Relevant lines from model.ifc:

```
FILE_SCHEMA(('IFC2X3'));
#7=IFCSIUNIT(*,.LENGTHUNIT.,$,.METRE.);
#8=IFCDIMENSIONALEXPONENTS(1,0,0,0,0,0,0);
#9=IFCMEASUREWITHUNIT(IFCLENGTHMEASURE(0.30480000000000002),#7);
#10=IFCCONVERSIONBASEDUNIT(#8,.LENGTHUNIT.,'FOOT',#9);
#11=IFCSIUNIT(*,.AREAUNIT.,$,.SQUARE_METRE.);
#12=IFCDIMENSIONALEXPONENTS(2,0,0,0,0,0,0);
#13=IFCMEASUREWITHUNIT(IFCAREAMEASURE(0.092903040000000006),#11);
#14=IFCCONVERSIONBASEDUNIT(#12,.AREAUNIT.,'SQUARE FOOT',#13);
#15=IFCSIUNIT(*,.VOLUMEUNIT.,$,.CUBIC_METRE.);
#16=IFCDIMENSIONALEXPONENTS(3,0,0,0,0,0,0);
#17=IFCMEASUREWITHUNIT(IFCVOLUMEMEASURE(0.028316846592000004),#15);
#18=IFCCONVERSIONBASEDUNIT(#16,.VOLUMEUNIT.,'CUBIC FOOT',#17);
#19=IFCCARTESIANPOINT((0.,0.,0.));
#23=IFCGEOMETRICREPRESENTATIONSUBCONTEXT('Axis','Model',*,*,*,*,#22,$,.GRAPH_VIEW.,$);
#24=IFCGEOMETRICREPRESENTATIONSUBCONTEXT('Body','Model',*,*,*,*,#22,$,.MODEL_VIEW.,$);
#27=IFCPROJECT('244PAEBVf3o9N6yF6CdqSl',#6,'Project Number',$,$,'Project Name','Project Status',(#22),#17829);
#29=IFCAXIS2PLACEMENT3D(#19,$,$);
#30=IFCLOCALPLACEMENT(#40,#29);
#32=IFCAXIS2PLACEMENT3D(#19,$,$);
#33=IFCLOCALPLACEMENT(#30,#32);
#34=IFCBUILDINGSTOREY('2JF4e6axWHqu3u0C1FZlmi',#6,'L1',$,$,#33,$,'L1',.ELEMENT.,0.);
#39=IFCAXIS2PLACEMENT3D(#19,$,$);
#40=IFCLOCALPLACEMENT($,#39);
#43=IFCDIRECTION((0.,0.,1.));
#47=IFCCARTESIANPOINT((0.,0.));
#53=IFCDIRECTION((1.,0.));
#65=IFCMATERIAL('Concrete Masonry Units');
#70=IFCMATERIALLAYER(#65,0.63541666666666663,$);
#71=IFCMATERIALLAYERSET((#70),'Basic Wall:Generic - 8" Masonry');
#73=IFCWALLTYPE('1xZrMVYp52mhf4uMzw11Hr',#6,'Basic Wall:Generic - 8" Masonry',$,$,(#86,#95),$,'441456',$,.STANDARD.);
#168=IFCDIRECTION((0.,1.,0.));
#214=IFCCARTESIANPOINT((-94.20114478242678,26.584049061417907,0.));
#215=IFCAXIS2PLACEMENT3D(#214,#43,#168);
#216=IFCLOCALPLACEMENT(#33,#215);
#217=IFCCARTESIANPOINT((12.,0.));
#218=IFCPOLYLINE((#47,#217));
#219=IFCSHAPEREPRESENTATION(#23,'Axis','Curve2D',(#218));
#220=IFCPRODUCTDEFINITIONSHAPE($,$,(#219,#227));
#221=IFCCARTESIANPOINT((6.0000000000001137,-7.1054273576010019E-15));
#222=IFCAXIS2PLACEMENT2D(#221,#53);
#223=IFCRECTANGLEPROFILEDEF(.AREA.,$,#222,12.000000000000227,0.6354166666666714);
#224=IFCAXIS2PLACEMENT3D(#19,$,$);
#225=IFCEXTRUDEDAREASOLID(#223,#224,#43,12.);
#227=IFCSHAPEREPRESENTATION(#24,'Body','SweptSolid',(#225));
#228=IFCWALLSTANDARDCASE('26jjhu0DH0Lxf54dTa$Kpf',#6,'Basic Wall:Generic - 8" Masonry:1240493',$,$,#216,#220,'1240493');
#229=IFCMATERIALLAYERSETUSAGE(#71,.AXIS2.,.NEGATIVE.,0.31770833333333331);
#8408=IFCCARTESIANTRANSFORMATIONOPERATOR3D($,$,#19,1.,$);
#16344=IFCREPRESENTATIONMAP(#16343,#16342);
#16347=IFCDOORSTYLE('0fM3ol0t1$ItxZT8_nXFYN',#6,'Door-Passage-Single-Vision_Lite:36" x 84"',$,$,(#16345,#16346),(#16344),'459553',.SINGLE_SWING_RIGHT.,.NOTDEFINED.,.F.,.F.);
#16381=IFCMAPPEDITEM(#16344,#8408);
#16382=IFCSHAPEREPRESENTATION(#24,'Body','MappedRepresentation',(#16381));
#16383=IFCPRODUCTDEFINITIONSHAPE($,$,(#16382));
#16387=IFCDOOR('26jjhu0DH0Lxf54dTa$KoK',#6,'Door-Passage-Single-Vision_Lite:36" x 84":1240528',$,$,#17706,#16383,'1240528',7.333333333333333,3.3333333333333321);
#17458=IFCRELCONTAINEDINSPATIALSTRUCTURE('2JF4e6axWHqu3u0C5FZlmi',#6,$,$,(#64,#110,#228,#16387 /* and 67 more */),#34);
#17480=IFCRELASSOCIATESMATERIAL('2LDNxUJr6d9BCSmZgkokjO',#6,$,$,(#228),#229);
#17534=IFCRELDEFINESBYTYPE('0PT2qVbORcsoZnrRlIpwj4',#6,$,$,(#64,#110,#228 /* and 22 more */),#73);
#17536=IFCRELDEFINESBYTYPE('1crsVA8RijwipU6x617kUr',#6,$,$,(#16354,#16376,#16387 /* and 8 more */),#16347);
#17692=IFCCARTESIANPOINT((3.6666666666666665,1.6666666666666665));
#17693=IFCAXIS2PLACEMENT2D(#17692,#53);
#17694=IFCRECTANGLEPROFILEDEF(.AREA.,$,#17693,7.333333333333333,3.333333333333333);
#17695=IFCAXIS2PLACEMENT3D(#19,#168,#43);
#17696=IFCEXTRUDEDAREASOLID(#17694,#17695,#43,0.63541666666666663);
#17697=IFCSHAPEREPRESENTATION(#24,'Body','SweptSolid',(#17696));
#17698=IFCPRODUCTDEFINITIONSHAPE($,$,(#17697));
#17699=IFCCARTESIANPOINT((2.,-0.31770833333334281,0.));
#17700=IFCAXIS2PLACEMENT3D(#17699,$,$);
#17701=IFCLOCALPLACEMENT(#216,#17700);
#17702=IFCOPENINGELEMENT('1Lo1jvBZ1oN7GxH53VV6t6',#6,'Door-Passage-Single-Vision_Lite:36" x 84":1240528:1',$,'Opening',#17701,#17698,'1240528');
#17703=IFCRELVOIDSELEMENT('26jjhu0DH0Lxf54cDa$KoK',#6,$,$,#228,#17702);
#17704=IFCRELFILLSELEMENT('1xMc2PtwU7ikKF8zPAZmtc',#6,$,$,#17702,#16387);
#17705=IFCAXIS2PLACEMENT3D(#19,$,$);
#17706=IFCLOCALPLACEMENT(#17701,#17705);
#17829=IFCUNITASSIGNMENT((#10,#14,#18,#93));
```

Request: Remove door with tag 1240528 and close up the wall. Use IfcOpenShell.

```python
import ifcopenshell
import ifcopenshell.api.feature
import ifcopenshell.api.root
import ifcopenshell.geom
import ifcopenshell.util.shape

model = ifcopenshell.open("model.ifc")
settings = ifcopenshell.geom.settings()


def volume(element):
    """Net volume in cubic metres, openings subtracted."""
    shape = ifcopenshell.geom.create_shape(settings, element)
    return ifcopenshell.util.shape.get_volume(shape.geometry)


door = model.by_guid("26jjhu0DH0Lxf54dTa$KoK")
opening = door.FillsVoids[0].RelatingOpeningElement
wall = opening.VoidsElements[0].RelatingBuildingElement
before = volume(wall)

ifcopenshell.api.root.remove_product(model, product=door)
ifcopenshell.api.feature.remove_feature(model, feature=opening)

after = volume(wall)

print(f"wall volume {before:.3f} -> {after:.3f} m3")

model.write("model_v2.ifc")
```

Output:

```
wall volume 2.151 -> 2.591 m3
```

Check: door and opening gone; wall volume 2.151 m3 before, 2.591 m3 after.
